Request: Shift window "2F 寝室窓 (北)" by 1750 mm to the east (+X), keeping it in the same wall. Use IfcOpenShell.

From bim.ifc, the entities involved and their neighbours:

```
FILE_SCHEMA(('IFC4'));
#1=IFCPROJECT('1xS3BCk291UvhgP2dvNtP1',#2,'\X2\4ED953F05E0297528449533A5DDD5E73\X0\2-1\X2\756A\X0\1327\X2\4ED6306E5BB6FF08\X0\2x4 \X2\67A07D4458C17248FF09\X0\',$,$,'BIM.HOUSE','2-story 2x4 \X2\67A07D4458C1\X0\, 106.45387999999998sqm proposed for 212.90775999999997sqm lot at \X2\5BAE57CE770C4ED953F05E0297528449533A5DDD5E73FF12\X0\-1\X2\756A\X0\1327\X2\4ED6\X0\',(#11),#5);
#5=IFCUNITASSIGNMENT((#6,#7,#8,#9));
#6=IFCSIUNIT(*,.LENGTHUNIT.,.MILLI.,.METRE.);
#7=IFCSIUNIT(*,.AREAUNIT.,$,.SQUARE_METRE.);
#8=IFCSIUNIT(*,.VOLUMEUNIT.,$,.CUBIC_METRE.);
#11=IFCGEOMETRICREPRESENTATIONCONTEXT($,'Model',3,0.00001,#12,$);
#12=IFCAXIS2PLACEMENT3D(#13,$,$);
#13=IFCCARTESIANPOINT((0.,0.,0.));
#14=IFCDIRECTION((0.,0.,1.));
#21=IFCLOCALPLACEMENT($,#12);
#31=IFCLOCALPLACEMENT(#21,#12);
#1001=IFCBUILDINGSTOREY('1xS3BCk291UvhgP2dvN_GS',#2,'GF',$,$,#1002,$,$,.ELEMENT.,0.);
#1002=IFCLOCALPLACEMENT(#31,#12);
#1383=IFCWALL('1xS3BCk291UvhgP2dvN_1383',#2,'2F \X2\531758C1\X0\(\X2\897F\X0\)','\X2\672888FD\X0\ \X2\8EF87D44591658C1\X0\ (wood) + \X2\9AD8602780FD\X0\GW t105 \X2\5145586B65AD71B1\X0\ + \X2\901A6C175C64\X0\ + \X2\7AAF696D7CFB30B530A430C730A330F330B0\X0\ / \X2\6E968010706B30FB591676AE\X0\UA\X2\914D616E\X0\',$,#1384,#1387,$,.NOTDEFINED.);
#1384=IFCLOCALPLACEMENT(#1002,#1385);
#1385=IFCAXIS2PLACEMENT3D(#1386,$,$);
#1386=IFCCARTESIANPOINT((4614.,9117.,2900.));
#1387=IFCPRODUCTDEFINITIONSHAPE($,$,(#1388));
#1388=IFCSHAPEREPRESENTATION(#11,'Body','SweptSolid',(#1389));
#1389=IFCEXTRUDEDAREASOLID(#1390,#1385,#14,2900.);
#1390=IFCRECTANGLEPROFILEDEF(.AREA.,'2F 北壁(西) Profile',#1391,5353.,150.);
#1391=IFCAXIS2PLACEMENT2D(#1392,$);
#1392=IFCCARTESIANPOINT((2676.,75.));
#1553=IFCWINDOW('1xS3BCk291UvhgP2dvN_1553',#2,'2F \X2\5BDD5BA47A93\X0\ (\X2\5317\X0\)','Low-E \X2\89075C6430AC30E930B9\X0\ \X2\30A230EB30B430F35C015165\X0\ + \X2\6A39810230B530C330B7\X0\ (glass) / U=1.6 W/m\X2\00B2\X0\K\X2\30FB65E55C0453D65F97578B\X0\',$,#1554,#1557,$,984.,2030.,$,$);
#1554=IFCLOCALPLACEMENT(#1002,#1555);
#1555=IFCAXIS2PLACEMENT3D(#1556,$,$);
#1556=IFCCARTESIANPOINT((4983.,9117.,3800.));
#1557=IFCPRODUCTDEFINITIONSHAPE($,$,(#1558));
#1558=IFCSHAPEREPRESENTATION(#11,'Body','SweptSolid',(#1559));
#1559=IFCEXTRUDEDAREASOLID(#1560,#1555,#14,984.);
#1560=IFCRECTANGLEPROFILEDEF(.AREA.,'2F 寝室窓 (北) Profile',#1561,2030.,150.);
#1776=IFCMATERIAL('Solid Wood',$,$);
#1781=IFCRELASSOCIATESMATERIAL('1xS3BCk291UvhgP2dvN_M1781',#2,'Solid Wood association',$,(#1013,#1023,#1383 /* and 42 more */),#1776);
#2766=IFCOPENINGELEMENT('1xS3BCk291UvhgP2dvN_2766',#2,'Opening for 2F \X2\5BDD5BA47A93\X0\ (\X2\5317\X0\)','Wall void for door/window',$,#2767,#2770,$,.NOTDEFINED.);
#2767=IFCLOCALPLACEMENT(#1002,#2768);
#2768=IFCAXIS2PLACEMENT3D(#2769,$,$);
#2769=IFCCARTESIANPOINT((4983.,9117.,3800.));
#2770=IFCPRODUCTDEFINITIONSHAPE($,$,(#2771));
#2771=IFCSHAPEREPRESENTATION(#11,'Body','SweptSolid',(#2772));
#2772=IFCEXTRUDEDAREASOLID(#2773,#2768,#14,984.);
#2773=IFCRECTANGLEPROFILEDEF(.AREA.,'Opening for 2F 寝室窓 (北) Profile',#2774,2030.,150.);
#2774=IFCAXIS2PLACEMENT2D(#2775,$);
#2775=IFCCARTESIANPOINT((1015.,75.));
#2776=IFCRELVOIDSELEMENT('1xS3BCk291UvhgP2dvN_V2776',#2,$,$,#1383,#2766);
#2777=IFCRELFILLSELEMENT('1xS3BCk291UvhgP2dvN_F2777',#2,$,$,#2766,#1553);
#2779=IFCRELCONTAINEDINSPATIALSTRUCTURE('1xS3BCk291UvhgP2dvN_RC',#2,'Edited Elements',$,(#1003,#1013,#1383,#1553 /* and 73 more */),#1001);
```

```python
import ifcopenshell
import ifcopenshell.api.geometry
import ifcopenshell.util.placement

model = ifcopenshell.open("bim.ifc")

window = model.by_guid("1xS3BCk291UvhgP2dvN_1553")
opening = window.FillsVoids[0].RelatingOpeningElement
wall = opening.VoidsElements[0].RelatingBuildingElement

wall_matrix = ifcopenshell.util.placement.get_local_placement(wall.ObjectPlacement)
shift = wall_matrix[:3, 0] * 1750.0
before = ifcopenshell.util.placement.get_local_placement(window.ObjectPlacement)[:3, 3].copy()

# The window is not placed relative to its opening, so move both.
for product in (opening, window):
    matrix = ifcopenshell.util.placement.get_local_placement(product.ObjectPlacement)
    matrix[:3, 3] += shift
    ifcopenshell.api.geometry.edit_object_placement(model, product=product, matrix=matrix, is_si=False)

after = ifcopenshell.util.placement.get_local_placement(window.ObjectPlacement)[:3, 3]
print("window moved by", (after - before).round(3) + 0.0)

model.write("bim_edited.ifc")
```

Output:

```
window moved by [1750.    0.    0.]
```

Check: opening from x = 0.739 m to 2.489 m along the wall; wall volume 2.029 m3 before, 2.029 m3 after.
